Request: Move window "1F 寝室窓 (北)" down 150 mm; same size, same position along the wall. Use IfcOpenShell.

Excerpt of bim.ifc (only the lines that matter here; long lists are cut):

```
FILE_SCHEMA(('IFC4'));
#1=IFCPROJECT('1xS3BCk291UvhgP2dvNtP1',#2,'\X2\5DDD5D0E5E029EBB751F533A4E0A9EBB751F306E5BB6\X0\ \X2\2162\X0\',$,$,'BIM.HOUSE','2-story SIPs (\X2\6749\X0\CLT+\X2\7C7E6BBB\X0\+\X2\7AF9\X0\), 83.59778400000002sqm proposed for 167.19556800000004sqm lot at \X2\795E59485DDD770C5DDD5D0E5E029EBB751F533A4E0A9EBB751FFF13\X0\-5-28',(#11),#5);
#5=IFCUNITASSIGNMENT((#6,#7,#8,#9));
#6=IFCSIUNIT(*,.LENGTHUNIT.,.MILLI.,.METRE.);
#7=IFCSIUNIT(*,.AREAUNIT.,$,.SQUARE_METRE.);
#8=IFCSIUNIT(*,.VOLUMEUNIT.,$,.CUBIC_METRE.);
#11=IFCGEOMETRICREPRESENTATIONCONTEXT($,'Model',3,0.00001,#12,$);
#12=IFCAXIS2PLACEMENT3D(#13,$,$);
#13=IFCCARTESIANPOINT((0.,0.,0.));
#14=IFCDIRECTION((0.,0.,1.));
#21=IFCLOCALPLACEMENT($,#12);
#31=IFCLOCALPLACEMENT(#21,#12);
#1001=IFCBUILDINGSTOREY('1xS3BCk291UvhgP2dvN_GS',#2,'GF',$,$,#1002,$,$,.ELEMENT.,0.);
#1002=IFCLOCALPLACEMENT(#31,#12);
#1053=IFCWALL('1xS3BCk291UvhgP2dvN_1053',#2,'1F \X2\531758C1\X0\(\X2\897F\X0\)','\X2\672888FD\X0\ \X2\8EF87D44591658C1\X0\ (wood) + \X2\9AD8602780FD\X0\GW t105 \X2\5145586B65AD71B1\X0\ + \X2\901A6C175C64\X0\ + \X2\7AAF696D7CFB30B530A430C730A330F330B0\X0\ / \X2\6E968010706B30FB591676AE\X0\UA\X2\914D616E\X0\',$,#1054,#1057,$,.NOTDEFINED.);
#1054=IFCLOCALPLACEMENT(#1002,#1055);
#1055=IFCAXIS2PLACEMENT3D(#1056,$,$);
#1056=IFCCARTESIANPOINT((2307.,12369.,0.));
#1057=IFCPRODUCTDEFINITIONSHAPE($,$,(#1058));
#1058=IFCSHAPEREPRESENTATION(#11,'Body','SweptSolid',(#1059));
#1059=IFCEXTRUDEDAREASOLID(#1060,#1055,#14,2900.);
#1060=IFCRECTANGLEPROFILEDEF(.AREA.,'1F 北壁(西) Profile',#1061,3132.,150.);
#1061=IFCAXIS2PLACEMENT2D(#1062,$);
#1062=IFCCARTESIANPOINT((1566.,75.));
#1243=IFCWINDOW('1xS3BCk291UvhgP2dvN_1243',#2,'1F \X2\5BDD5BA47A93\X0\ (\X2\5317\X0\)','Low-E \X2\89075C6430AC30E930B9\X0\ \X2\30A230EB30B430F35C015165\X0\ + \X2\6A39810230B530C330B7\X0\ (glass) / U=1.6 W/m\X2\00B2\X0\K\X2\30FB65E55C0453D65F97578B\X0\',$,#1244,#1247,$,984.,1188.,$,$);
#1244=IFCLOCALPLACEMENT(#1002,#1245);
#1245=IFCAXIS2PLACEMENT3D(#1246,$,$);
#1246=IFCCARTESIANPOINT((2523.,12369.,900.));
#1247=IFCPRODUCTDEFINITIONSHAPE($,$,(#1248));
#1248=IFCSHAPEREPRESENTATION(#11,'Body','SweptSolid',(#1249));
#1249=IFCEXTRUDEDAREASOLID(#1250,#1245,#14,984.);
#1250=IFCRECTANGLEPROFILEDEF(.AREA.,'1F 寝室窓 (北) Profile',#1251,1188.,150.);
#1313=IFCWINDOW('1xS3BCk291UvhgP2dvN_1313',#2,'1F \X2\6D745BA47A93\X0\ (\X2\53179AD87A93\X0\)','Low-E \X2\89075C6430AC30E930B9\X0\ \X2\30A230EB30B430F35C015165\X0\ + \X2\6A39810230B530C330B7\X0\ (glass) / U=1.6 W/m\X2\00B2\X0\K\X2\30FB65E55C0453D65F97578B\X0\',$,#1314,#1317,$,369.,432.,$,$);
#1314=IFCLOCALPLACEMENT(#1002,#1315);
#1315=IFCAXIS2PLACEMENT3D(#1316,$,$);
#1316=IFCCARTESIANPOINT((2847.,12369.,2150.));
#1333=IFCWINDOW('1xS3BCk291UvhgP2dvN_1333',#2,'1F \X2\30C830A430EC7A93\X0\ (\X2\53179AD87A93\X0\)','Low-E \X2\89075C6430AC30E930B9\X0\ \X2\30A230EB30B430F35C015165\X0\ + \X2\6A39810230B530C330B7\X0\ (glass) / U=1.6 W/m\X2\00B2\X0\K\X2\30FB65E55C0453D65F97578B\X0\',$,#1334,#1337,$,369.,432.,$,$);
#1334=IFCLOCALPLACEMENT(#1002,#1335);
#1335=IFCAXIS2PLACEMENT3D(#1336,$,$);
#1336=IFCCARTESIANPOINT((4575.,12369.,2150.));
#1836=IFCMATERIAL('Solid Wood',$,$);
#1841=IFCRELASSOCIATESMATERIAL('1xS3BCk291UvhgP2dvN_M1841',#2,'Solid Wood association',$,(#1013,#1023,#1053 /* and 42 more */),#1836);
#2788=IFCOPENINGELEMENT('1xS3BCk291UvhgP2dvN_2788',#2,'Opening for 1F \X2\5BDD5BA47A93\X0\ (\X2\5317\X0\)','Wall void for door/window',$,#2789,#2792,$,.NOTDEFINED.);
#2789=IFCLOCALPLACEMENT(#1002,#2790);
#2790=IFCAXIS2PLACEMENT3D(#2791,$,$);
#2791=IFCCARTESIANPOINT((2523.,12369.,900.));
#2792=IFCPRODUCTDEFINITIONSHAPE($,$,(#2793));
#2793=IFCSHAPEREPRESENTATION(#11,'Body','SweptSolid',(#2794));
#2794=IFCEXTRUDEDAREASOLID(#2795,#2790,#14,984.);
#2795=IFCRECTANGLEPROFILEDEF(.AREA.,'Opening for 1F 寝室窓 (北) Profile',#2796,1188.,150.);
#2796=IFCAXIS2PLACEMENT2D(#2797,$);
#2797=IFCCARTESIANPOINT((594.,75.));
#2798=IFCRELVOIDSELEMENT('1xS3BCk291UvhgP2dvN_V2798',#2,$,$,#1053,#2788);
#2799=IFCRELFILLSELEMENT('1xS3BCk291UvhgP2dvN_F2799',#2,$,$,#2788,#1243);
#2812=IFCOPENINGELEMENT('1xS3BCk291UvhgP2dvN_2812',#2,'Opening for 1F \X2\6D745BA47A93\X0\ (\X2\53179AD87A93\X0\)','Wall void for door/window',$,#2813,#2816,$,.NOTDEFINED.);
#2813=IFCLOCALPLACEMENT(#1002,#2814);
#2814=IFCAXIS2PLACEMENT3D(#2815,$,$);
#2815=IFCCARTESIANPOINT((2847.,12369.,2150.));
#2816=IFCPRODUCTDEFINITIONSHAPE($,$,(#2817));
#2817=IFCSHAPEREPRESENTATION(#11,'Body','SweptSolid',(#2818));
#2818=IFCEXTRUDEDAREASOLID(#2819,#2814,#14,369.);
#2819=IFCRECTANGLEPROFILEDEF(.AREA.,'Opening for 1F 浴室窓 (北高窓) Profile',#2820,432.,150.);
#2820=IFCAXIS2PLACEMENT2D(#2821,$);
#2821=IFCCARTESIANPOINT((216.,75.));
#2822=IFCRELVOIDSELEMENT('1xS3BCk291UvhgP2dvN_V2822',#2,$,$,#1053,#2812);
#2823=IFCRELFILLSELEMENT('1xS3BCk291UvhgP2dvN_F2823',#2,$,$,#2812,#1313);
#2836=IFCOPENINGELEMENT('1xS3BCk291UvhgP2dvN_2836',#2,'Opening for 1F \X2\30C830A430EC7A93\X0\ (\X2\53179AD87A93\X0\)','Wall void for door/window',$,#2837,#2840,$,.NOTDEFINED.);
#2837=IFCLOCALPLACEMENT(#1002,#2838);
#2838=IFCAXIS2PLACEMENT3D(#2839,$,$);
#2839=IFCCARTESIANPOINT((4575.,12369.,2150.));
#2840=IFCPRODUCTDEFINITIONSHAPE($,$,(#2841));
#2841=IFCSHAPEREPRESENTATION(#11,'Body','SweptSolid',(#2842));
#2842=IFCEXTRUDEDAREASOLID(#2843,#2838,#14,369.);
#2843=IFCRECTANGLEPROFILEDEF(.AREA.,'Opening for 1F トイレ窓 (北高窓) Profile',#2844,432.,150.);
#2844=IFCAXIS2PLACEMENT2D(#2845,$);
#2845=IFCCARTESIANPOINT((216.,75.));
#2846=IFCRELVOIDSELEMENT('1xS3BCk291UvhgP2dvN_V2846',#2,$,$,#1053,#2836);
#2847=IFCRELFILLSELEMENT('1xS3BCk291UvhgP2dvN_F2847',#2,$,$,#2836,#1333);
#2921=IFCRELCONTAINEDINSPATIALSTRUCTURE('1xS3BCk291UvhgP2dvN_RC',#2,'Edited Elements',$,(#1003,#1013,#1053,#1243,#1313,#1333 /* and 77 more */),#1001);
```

```python
import numpy as np
import ifcopenshell
import ifcopenshell.api.geometry
import ifcopenshell.util.placement
import ifcopenshell.util.unit

model = ifcopenshell.open("bim.ifc")
unit_scale = ifcopenshell.util.unit.calculate_unit_scale(model)

window = model.by_guid("1xS3BCk291UvhgP2dvN_1243")
opening = window.FillsVoids[0].RelatingOpeningElement
dz = -0.15 / unit_scale

shift = np.array([0.0, 0.0, dz])
# The window is not placed relative to its opening, so move both.
for product in (opening, window):
    matrix = ifcopenshell.util.placement.get_local_placement(product.ObjectPlacement)
    matrix[:3, 3] += shift
    ifcopenshell.api.geometry.edit_object_placement(model, product=product, matrix=matrix, is_si=False)

print(f"moved by {dz * unit_scale:+.3f} m")

model.write("bim_updated.ifc")
```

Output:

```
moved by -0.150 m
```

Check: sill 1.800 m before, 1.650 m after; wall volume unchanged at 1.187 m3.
